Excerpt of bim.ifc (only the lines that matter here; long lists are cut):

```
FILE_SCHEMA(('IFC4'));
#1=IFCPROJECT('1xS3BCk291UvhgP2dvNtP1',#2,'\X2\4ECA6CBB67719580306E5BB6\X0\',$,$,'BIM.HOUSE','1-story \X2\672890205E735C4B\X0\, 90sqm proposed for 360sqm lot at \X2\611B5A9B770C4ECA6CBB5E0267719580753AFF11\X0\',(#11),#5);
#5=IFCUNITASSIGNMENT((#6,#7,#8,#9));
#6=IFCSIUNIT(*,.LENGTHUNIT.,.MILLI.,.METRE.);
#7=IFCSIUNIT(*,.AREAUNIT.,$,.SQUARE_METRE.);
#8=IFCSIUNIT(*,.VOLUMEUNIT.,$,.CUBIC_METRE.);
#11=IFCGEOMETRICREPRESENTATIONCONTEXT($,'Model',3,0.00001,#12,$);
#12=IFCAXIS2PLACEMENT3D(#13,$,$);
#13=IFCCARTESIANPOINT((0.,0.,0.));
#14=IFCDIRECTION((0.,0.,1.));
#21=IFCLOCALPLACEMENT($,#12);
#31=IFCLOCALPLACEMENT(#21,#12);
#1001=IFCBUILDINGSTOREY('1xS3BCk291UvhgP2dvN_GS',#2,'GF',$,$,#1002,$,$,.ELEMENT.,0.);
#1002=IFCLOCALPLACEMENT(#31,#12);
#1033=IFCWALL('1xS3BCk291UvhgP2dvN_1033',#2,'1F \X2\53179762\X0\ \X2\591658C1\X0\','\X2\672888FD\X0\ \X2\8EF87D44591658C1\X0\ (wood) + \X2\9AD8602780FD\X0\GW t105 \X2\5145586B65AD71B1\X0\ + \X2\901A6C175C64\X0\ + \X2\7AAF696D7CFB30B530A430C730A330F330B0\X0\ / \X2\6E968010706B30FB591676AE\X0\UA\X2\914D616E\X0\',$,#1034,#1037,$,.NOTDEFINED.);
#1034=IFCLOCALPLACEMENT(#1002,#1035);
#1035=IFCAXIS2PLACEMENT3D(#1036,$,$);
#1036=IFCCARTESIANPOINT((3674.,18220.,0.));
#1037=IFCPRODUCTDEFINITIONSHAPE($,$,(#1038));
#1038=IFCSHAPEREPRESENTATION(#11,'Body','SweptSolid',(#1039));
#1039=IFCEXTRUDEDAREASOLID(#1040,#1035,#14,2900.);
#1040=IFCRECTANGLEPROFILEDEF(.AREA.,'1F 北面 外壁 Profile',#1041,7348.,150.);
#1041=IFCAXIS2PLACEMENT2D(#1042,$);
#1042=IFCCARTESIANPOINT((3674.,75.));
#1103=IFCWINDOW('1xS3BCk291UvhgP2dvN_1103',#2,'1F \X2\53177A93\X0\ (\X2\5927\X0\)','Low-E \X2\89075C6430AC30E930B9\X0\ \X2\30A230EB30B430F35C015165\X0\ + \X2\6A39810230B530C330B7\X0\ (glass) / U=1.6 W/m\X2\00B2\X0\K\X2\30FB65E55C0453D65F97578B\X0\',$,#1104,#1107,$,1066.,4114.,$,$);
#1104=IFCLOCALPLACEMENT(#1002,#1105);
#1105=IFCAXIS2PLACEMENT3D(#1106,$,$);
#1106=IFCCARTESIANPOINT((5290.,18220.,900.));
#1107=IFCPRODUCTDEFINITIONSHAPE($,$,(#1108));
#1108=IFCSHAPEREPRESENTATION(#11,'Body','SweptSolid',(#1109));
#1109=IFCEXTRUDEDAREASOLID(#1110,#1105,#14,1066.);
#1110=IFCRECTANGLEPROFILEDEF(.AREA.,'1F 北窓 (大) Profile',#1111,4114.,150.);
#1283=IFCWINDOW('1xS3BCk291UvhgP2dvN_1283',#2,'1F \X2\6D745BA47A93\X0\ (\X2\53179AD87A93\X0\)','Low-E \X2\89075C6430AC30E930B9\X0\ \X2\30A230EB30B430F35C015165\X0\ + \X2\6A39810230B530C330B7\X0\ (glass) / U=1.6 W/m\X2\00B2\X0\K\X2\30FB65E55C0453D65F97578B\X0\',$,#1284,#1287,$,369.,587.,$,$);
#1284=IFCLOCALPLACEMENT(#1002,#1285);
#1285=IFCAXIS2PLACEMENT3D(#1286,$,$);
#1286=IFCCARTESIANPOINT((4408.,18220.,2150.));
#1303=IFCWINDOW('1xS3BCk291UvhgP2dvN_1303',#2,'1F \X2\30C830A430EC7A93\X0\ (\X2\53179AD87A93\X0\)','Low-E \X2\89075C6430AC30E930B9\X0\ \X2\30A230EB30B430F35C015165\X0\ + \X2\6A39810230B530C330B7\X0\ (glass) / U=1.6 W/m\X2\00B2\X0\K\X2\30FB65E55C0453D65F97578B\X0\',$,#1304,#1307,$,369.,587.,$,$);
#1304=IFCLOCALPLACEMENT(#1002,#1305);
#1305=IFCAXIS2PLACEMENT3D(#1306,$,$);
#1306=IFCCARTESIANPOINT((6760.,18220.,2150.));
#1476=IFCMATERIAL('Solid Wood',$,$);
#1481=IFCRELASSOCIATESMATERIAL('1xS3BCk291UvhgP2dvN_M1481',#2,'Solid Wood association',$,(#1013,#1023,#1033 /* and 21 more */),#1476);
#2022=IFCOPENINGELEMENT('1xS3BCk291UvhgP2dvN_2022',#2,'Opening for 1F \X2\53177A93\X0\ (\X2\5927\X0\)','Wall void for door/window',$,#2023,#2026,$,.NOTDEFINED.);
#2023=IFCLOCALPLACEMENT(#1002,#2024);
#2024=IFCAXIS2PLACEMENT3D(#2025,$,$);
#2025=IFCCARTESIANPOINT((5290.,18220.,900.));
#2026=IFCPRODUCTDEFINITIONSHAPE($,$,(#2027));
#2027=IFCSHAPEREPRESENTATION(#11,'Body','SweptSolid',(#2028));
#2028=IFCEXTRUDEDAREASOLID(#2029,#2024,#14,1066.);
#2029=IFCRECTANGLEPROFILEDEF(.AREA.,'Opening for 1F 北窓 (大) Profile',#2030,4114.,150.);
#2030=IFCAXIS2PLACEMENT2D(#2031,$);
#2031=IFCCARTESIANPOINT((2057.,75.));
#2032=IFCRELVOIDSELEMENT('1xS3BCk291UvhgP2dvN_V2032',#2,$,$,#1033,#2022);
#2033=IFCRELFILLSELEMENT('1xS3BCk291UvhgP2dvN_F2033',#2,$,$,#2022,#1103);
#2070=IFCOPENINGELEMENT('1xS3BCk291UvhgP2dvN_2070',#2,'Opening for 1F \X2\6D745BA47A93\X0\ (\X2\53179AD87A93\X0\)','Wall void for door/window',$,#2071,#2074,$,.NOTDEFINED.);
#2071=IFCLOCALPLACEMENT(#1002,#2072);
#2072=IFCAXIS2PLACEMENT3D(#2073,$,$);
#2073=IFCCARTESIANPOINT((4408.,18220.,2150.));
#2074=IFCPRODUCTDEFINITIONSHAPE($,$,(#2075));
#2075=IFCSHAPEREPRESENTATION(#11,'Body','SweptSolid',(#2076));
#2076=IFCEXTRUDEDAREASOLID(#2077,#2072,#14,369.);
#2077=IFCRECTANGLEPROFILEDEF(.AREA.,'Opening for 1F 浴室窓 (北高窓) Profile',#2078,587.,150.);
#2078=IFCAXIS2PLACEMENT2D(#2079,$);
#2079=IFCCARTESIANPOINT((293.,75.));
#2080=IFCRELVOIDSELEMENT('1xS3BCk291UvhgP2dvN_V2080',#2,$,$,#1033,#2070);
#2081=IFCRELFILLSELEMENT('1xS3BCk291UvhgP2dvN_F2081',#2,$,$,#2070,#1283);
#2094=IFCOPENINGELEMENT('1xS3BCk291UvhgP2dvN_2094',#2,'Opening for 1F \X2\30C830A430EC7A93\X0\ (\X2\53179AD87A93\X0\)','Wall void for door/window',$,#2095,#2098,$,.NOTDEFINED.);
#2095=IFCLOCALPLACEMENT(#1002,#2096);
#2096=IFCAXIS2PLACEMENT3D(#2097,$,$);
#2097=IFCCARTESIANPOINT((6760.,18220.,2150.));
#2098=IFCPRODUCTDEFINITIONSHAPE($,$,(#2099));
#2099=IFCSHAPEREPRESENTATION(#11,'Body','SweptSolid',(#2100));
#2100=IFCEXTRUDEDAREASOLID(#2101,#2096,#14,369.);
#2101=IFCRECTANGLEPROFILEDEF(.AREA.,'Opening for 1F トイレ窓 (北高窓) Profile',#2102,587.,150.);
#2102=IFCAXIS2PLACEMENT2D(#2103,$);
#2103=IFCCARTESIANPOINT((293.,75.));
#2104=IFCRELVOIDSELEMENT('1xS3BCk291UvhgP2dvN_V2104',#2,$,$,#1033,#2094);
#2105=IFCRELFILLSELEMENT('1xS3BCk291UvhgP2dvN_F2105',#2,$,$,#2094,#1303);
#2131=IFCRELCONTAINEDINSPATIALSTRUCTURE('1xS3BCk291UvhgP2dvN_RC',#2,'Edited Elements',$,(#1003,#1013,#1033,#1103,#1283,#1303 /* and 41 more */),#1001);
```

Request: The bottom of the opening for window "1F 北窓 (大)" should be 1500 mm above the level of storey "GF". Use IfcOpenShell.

```python
import numpy as np
import ifcopenshell
import ifcopenshell.api.geometry
import ifcopenshell.geom
import ifcopenshell.util.element
import ifcopenshell.util.placement
import ifcopenshell.util.shape
import ifcopenshell.util.unit

model = ifcopenshell.open("bim.ifc")
unit_scale = ifcopenshell.util.unit.calculate_unit_scale(model)

window = model.by_guid("1xS3BCk291UvhgP2dvN_1103")
opening = window.FillsVoids[0].RelatingOpeningElement
storey = ifcopenshell.util.element.get_container(window, ifc_class="IfcBuildingStorey")
level = ifcopenshell.util.placement.get_local_placement(storey.ObjectPlacement)[2, 3]

# The opening's origin need not be at the sill, so measure its lowest point.
shape = ifcopenshell.geom.create_shape(ifcopenshell.geom.settings(), opening)
bottom = ifcopenshell.util.shape.get_shape_bottom_elevation(shape, shape.geometry) / unit_scale
dz = level + 1500.0 - bottom

shift = np.array([0.0, 0.0, dz])
# The window is not placed relative to its opening, so move both.
for product in (opening, window):
    matrix = ifcopenshell.util.placement.get_local_placement(product.ObjectPlacement)
    matrix[:3, 3] += shift
    ifcopenshell.api.geometry.edit_object_placement(model, product=product, matrix=matrix, is_si=False)

print(f"moved by {dz * unit_scale:+.3f} m")

model.write("bim_edited.ifc")
```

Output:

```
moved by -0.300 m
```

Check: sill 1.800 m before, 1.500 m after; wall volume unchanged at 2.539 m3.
